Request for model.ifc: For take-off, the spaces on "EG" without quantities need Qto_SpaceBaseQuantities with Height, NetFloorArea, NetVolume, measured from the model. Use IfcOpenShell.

First a look at what the model holds.

```python
import ifcopenshell
import ifcopenshell.util.element
import ifcopenshell.util.unit

model = ifcopenshell.open("model.ifc")
print(model.schema)
for unit_type in ("LENGTHUNIT", "AREAUNIT", "VOLUMEUNIT"):
    print(unit_type, ifcopenshell.util.unit.calculate_unit_scale(model, unit_type))
storey = next(s for s in model.by_type("IfcBuildingStorey") if s.Name == "EG")
spaces = [e for e in ifcopenshell.util.element.get_decomposition(storey) if e.is_a("IfcSpace")]
for e in sorted(spaces, key=lambda e: e.id()):
    print(e.id(), e.is_a(), e.Name, list(ifcopenshell.util.element.get_psets(e, qtos_only=True)), sep=" | ")
```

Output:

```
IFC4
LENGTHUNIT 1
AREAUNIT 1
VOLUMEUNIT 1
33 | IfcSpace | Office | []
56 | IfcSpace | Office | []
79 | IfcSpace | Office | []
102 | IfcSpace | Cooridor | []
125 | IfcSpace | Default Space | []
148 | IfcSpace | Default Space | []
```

```python
import ifcopenshell
import ifcopenshell.api.pset
import ifcopenshell.geom
import ifcopenshell.util.element
import ifcopenshell.util.shape
import ifcopenshell.util.unit

model = ifcopenshell.open("model.ifc")
unit_scale = ifcopenshell.util.unit.calculate_unit_scale(model)
area_scale = ifcopenshell.util.unit.calculate_unit_scale(model, "AREAUNIT")
volume_scale = ifcopenshell.util.unit.calculate_unit_scale(model, "VOLUMEUNIT")
settings = ifcopenshell.geom.settings()

storey = next(s for s in model.by_type("IfcBuildingStorey") if s.Name == "EG")
spaces = [e for e in ifcopenshell.util.element.get_decomposition(storey) if e.is_a("IfcSpace")]

for e in sorted(spaces, key=lambda e: e.id()):
    if ifcopenshell.util.element.get_psets(e, qtos_only=True, should_inherit=False):
        continue
    # Geometry comes back in metres, in the element's own axes.
    shape = ifcopenshell.geom.create_shape(settings, e)
    values = {
        "Height": ifcopenshell.util.shape.get_z(shape.geometry) / unit_scale,
        "NetFloorArea": ifcopenshell.util.shape.get_footprint_area(shape.geometry) / area_scale,
        "NetVolume": ifcopenshell.util.shape.get_volume(shape.geometry) / volume_scale,
    }
    qto = ifcopenshell.api.pset.add_qto(model, product=e, name="Qto_SpaceBaseQuantities")
    ifcopenshell.api.pset.edit_qto(model, qto=qto, properties=values)
    print(e.id(), {k: round(v, 3) for k, v in values.items()})

model.write("model_v2.ifc")
```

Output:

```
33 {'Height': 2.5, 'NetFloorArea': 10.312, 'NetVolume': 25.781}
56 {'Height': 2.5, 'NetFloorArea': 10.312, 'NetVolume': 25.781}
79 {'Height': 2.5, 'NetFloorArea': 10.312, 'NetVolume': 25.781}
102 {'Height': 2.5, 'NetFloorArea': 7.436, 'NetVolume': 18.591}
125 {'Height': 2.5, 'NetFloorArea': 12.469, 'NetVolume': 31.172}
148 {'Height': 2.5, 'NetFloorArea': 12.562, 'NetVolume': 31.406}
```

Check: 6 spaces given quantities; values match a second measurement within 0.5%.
